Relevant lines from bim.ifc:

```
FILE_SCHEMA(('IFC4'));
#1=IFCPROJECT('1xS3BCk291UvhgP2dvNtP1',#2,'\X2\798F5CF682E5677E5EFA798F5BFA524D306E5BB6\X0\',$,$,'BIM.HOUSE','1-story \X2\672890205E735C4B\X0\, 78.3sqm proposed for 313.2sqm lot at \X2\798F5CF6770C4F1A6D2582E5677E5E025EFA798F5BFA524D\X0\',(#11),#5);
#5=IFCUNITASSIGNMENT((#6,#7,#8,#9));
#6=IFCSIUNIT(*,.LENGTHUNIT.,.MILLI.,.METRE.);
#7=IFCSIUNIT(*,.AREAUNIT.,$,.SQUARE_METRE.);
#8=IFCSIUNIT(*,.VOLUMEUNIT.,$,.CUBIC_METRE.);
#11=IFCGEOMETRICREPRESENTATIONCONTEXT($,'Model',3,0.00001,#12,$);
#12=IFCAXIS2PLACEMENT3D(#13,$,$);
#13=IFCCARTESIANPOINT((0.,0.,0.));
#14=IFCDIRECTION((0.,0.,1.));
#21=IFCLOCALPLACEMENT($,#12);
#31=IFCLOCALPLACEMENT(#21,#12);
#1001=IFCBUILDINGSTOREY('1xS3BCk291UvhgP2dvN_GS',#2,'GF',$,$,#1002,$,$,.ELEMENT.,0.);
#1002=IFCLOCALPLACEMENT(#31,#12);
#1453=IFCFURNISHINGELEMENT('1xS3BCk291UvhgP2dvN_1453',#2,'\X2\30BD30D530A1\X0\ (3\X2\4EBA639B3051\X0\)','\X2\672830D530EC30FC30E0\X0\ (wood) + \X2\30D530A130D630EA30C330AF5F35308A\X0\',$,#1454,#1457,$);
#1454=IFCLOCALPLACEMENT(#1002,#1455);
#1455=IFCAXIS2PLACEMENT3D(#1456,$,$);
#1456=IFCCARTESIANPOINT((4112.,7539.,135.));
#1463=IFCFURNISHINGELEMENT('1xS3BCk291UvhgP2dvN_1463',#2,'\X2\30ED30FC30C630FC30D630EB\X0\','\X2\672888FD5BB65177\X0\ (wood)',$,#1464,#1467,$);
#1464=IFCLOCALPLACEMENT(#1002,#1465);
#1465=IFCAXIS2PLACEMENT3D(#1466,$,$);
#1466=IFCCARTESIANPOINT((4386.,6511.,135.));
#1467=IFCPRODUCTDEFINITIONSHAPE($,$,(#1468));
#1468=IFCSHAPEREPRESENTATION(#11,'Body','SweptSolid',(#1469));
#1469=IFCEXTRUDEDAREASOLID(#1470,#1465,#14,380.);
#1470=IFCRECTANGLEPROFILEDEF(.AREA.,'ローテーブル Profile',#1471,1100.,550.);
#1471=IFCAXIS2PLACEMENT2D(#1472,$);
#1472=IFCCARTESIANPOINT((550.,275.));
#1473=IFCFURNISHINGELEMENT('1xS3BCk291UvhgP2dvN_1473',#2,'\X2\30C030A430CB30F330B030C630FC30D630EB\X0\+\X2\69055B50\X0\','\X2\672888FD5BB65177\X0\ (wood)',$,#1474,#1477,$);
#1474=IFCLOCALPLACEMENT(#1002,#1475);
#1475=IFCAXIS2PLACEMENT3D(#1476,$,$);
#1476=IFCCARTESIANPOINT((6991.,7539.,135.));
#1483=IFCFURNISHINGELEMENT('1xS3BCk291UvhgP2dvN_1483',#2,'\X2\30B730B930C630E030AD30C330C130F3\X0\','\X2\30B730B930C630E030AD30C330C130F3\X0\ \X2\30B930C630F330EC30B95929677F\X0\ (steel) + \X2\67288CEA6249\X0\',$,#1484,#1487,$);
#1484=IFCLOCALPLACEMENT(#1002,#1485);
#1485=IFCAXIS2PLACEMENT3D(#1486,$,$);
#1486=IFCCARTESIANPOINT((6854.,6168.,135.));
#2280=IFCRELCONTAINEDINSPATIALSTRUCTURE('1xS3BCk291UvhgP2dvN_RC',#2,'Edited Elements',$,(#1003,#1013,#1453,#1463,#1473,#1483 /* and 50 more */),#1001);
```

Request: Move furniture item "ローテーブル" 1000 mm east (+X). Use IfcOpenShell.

```python
import ifcopenshell
import ifcopenshell.api.geometry
import ifcopenshell.util.placement

model = ifcopenshell.open("bim.ifc")

item = model.by_guid("1xS3BCk291UvhgP2dvN_1463")
matrix = ifcopenshell.util.placement.get_local_placement(item.ObjectPlacement)
matrix[0, 3] += 1000.0
ifcopenshell.api.geometry.edit_object_placement(model, product=item, matrix=matrix, is_si=False)

print(ifcopenshell.util.placement.get_local_placement(item.ObjectPlacement).round(3) + 0.0)

model.write("bim-out.ifc")
```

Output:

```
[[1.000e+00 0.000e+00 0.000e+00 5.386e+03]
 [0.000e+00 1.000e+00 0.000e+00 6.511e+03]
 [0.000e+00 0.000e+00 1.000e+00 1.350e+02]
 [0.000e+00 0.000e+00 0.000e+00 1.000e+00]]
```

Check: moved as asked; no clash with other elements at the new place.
